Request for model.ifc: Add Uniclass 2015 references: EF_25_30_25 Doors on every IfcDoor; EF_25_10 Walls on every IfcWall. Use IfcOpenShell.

First a look at what the model holds.

```python
import ifcopenshell

model = ifcopenshell.open("model.ifc")
print(model.schema)
print("classifications:", [c.Name for c in model.by_type("IfcClassification")])
for ifc_class in ("IfcDoor", "IfcRoof", "IfcStair", "IfcWall", "IfcWindow"):
    print(ifc_class, len(model.by_type(ifc_class)))
```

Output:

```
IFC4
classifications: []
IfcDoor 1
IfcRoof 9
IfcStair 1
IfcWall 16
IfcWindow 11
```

```python
import ifcopenshell
import ifcopenshell.api.classification

model = ifcopenshell.open("model.ifc")

system = ifcopenshell.api.classification.add_classification(model, classification="Uniclass 2015")

codes = {
    "IfcDoor": ("EF_25_30_25", "Doors"),
    "IfcWall": ("EF_25_10", "Walls"),
}
for ifc_class, (code, name) in codes.items():
    products = model.by_type(ifc_class)
    ifcopenshell.api.classification.add_reference(
        model, products=products, classification=system, identification=code, name=name
    )
    print(code, len(products))

model.write("model-out.ifc")
```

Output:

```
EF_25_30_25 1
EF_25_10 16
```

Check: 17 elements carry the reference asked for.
